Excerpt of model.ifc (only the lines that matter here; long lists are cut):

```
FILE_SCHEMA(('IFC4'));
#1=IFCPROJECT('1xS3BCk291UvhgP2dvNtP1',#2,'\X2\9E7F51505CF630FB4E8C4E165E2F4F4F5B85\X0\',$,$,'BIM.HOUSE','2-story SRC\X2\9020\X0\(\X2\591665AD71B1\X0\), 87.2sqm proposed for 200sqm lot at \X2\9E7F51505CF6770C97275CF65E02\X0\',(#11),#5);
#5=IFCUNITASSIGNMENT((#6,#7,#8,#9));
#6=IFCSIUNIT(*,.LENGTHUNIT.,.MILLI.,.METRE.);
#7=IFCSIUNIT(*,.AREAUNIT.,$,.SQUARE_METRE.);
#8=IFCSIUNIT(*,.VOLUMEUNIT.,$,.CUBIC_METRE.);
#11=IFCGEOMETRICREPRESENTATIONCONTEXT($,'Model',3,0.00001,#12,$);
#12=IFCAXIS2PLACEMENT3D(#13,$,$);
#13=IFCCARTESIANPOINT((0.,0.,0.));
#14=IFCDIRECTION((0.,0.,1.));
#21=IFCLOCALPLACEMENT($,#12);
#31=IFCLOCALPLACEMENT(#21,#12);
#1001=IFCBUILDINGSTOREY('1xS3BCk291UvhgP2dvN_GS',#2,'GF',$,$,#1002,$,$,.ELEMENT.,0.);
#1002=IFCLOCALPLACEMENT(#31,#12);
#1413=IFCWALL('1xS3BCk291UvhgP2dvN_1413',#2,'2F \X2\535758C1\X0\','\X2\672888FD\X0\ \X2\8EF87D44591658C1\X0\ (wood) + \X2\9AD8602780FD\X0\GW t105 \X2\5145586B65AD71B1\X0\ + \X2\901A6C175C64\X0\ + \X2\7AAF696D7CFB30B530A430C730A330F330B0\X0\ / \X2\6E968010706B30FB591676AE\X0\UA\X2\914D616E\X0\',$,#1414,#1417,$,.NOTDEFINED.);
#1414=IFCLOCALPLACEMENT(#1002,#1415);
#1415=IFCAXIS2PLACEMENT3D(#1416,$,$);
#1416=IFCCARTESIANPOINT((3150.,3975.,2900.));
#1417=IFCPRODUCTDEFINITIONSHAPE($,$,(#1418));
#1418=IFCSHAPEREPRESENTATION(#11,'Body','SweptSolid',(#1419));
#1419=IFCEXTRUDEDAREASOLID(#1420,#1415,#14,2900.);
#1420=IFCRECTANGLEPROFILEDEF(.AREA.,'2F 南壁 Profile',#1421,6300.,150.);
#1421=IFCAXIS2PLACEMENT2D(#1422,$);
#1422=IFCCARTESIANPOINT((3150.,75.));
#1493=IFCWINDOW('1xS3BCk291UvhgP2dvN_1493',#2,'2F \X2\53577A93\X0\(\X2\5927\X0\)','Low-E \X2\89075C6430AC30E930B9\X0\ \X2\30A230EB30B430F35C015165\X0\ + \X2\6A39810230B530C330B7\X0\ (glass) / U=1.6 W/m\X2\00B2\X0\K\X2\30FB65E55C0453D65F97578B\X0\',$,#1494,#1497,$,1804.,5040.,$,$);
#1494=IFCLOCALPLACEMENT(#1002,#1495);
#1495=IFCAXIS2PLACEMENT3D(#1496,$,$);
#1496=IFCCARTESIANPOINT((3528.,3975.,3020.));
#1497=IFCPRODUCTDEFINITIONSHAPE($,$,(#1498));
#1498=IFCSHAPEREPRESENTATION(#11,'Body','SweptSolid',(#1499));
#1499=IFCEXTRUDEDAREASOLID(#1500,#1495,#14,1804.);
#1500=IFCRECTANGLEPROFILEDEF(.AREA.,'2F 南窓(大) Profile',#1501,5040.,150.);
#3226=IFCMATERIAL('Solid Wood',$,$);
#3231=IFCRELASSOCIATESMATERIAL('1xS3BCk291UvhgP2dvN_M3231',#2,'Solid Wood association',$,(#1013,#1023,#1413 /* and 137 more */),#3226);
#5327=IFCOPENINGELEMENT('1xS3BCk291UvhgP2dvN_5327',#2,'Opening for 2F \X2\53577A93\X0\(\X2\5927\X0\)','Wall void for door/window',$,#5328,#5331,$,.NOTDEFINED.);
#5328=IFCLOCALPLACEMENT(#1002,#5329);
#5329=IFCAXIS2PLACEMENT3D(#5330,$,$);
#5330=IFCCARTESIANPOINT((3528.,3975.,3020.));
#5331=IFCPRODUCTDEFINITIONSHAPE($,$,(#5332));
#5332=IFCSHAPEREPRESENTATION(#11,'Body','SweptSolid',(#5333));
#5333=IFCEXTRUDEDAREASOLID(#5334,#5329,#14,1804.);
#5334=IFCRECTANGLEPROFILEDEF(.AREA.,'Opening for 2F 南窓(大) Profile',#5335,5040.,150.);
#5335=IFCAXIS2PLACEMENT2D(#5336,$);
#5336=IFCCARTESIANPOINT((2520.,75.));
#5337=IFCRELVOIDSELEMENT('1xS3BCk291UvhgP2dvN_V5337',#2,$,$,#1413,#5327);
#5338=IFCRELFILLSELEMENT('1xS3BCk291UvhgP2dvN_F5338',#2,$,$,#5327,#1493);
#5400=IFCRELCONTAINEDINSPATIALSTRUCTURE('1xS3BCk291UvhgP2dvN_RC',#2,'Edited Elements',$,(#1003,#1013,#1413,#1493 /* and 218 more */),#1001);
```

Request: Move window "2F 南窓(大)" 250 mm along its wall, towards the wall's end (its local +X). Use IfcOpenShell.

```python
import ifcopenshell
import ifcopenshell.api.geometry
import ifcopenshell.util.placement

model = ifcopenshell.open("model.ifc")

window = model.by_id(1493)
opening = window.FillsVoids[0].RelatingOpeningElement
wall = opening.VoidsElements[0].RelatingBuildingElement

wall_matrix = ifcopenshell.util.placement.get_local_placement(wall.ObjectPlacement)
shift = wall_matrix[:3, 0] * 250.0
before = ifcopenshell.util.placement.get_local_placement(window.ObjectPlacement)[:3, 3].copy()

# The window is not placed relative to its opening, so move both.
for product in (opening, window):
    matrix = ifcopenshell.util.placement.get_local_placement(product.ObjectPlacement)
    matrix[:3, 3] += shift
    ifcopenshell.api.geometry.edit_object_placement(model, product=product, matrix=matrix, is_si=False)

after = ifcopenshell.util.placement.get_local_placement(window.ObjectPlacement)[:3, 3]
print("window moved by", (after - before).round(3) + 0.0)

model.write("model_updated.ifc")
```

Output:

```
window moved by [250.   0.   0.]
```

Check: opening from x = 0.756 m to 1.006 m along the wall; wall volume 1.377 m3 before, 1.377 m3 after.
